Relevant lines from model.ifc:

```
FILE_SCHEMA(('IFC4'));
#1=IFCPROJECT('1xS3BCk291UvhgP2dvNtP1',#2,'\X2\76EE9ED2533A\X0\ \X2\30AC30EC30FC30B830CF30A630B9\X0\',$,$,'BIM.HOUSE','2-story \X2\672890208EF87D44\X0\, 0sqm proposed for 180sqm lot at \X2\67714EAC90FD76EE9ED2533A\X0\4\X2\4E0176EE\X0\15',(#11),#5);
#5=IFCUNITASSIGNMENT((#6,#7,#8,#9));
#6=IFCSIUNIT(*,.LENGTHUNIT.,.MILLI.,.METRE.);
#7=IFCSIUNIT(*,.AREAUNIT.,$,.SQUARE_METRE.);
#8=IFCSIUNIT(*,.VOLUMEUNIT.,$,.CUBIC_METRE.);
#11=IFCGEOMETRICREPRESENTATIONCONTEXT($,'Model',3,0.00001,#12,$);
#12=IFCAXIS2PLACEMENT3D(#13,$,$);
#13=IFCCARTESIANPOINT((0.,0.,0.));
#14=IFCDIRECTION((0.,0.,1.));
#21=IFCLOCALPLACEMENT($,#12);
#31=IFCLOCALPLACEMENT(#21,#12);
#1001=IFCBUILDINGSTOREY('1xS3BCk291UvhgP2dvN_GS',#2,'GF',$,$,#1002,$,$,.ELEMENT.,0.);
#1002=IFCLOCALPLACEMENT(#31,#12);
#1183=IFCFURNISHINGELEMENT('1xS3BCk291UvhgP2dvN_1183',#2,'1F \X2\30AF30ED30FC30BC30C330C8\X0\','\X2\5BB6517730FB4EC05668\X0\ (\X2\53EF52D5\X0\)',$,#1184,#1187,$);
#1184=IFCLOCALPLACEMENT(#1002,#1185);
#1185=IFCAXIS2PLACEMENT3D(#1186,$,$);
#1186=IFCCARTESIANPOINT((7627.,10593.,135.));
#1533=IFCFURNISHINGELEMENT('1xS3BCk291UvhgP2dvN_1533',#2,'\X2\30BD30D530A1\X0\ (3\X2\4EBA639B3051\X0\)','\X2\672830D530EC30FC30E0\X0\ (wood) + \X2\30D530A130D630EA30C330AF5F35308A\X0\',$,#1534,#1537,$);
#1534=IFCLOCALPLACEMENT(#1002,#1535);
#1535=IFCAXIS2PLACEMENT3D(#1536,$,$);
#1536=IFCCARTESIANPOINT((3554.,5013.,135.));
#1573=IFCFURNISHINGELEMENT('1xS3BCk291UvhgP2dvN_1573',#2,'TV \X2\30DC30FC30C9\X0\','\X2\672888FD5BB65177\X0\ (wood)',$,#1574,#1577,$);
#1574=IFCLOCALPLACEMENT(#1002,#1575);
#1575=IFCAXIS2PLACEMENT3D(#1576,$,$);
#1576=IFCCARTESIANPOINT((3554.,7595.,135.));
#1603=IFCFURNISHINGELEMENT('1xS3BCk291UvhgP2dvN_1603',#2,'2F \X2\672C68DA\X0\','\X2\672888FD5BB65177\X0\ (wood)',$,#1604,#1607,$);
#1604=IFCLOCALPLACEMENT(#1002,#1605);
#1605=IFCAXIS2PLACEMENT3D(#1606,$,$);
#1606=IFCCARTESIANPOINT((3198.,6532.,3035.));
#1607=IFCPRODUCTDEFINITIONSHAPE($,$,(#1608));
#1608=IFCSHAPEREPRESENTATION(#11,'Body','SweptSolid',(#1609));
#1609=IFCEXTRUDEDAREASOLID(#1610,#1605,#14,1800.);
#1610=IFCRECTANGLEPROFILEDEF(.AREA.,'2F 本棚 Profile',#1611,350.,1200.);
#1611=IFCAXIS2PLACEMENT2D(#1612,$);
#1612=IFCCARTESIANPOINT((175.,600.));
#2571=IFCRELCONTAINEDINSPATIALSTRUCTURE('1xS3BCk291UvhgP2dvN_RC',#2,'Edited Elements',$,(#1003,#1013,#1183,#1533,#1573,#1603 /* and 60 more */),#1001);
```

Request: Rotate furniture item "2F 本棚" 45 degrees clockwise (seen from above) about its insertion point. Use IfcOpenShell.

```python
import ifcopenshell
import ifcopenshell.api.geometry
import ifcopenshell.util.placement

model = ifcopenshell.open("model.ifc")

item = model.by_id(1603)
matrix = ifcopenshell.util.placement.get_local_placement(item.ObjectPlacement)
matrix = matrix @ ifcopenshell.util.placement.rotation(-45, "Z")
ifcopenshell.api.geometry.edit_object_placement(model, product=item, matrix=matrix, is_si=False)

print(ifcopenshell.util.placement.get_local_placement(item.ObjectPlacement).round(3) + 0.0)

model.write("model-out.ifc")
```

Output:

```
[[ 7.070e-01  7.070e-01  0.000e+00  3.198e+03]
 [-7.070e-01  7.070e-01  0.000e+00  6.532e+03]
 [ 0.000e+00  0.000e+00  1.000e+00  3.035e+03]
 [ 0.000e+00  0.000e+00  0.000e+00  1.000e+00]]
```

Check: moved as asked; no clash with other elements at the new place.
